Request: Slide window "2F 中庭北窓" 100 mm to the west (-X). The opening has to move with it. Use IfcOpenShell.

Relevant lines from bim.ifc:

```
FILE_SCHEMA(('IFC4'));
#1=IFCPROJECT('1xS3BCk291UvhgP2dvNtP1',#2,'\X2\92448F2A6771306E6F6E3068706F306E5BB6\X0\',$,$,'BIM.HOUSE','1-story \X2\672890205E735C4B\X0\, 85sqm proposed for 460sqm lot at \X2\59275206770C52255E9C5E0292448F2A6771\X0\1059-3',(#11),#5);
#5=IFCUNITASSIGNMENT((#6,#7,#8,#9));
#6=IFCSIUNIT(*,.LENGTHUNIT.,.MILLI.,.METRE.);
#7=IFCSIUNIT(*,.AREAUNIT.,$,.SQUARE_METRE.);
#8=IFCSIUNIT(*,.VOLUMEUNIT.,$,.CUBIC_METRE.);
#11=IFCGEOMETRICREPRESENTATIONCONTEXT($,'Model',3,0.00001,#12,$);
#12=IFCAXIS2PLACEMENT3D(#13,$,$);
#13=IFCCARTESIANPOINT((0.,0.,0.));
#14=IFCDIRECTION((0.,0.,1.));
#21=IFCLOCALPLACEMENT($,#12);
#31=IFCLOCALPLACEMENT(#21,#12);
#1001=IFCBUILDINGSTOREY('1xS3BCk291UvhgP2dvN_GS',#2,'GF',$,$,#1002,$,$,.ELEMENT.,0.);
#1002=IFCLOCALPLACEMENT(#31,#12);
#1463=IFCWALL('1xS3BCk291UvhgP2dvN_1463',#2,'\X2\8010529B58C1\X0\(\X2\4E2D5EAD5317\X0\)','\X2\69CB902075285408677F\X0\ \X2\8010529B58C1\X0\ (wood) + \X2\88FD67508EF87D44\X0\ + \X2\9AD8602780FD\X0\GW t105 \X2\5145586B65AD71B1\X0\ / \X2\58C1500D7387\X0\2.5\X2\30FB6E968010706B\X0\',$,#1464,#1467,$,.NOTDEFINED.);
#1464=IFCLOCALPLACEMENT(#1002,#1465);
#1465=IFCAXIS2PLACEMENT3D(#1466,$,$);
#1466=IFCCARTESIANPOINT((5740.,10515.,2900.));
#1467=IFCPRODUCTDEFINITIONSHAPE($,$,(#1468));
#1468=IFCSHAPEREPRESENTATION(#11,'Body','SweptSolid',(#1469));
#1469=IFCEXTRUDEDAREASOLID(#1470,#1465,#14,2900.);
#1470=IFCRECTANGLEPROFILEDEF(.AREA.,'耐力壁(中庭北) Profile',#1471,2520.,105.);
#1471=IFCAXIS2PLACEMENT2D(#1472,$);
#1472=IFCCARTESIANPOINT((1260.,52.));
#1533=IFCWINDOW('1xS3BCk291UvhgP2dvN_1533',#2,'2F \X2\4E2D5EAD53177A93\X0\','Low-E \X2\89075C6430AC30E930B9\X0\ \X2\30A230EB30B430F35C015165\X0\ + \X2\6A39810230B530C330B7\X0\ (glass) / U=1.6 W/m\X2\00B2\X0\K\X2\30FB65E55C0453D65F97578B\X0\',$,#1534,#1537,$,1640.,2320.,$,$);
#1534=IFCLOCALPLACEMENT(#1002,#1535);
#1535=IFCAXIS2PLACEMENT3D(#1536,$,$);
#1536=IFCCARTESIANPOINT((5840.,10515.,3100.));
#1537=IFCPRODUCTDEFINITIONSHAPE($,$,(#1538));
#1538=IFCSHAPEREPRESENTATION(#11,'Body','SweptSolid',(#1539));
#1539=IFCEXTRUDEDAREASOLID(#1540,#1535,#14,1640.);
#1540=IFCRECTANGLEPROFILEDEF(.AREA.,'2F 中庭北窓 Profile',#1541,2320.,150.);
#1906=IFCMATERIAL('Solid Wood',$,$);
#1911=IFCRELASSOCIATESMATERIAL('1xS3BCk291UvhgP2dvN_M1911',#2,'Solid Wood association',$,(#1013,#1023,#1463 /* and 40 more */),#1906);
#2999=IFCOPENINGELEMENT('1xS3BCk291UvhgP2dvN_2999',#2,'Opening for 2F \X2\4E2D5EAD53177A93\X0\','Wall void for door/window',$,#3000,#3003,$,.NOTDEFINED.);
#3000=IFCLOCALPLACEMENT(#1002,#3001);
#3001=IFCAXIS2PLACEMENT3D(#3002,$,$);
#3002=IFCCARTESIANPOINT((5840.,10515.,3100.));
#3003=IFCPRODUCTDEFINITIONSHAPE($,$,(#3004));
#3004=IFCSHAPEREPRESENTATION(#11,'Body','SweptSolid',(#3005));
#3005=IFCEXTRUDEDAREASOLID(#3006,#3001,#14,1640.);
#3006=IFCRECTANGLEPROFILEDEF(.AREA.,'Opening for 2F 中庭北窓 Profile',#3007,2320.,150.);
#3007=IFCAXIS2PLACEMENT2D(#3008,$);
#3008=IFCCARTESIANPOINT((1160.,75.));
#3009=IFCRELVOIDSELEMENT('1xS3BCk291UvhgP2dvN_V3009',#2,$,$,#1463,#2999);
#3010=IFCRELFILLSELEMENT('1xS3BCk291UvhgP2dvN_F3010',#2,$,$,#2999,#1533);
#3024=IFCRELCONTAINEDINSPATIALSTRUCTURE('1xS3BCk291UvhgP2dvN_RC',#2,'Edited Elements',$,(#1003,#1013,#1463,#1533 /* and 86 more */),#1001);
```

```python
import ifcopenshell
import ifcopenshell.api.geometry
import ifcopenshell.util.placement

model = ifcopenshell.open("bim.ifc")

window = model.by_guid("1xS3BCk291UvhgP2dvN_1533")
opening = window.FillsVoids[0].RelatingOpeningElement
wall = opening.VoidsElements[0].RelatingBuildingElement

wall_matrix = ifcopenshell.util.placement.get_local_placement(wall.ObjectPlacement)
shift = wall_matrix[:3, 0] * -100.0
before = ifcopenshell.util.placement.get_local_placement(window.ObjectPlacement)[:3, 3].copy()

# The window is not placed relative to its opening, so move both.
for product in (opening, window):
    matrix = ifcopenshell.util.placement.get_local_placement(product.ObjectPlacement)
    matrix[:3, 3] += shift
    ifcopenshell.api.geometry.edit_object_placement(model, product=product, matrix=matrix, is_si=False)

after = ifcopenshell.util.placement.get_local_placement(window.ObjectPlacement)[:3, 3]
print("window moved by", (after - before).round(3) + 0.0)

model.write("bim_edited.ifc")
```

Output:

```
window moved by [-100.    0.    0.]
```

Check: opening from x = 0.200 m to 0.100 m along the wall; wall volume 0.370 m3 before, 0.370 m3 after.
